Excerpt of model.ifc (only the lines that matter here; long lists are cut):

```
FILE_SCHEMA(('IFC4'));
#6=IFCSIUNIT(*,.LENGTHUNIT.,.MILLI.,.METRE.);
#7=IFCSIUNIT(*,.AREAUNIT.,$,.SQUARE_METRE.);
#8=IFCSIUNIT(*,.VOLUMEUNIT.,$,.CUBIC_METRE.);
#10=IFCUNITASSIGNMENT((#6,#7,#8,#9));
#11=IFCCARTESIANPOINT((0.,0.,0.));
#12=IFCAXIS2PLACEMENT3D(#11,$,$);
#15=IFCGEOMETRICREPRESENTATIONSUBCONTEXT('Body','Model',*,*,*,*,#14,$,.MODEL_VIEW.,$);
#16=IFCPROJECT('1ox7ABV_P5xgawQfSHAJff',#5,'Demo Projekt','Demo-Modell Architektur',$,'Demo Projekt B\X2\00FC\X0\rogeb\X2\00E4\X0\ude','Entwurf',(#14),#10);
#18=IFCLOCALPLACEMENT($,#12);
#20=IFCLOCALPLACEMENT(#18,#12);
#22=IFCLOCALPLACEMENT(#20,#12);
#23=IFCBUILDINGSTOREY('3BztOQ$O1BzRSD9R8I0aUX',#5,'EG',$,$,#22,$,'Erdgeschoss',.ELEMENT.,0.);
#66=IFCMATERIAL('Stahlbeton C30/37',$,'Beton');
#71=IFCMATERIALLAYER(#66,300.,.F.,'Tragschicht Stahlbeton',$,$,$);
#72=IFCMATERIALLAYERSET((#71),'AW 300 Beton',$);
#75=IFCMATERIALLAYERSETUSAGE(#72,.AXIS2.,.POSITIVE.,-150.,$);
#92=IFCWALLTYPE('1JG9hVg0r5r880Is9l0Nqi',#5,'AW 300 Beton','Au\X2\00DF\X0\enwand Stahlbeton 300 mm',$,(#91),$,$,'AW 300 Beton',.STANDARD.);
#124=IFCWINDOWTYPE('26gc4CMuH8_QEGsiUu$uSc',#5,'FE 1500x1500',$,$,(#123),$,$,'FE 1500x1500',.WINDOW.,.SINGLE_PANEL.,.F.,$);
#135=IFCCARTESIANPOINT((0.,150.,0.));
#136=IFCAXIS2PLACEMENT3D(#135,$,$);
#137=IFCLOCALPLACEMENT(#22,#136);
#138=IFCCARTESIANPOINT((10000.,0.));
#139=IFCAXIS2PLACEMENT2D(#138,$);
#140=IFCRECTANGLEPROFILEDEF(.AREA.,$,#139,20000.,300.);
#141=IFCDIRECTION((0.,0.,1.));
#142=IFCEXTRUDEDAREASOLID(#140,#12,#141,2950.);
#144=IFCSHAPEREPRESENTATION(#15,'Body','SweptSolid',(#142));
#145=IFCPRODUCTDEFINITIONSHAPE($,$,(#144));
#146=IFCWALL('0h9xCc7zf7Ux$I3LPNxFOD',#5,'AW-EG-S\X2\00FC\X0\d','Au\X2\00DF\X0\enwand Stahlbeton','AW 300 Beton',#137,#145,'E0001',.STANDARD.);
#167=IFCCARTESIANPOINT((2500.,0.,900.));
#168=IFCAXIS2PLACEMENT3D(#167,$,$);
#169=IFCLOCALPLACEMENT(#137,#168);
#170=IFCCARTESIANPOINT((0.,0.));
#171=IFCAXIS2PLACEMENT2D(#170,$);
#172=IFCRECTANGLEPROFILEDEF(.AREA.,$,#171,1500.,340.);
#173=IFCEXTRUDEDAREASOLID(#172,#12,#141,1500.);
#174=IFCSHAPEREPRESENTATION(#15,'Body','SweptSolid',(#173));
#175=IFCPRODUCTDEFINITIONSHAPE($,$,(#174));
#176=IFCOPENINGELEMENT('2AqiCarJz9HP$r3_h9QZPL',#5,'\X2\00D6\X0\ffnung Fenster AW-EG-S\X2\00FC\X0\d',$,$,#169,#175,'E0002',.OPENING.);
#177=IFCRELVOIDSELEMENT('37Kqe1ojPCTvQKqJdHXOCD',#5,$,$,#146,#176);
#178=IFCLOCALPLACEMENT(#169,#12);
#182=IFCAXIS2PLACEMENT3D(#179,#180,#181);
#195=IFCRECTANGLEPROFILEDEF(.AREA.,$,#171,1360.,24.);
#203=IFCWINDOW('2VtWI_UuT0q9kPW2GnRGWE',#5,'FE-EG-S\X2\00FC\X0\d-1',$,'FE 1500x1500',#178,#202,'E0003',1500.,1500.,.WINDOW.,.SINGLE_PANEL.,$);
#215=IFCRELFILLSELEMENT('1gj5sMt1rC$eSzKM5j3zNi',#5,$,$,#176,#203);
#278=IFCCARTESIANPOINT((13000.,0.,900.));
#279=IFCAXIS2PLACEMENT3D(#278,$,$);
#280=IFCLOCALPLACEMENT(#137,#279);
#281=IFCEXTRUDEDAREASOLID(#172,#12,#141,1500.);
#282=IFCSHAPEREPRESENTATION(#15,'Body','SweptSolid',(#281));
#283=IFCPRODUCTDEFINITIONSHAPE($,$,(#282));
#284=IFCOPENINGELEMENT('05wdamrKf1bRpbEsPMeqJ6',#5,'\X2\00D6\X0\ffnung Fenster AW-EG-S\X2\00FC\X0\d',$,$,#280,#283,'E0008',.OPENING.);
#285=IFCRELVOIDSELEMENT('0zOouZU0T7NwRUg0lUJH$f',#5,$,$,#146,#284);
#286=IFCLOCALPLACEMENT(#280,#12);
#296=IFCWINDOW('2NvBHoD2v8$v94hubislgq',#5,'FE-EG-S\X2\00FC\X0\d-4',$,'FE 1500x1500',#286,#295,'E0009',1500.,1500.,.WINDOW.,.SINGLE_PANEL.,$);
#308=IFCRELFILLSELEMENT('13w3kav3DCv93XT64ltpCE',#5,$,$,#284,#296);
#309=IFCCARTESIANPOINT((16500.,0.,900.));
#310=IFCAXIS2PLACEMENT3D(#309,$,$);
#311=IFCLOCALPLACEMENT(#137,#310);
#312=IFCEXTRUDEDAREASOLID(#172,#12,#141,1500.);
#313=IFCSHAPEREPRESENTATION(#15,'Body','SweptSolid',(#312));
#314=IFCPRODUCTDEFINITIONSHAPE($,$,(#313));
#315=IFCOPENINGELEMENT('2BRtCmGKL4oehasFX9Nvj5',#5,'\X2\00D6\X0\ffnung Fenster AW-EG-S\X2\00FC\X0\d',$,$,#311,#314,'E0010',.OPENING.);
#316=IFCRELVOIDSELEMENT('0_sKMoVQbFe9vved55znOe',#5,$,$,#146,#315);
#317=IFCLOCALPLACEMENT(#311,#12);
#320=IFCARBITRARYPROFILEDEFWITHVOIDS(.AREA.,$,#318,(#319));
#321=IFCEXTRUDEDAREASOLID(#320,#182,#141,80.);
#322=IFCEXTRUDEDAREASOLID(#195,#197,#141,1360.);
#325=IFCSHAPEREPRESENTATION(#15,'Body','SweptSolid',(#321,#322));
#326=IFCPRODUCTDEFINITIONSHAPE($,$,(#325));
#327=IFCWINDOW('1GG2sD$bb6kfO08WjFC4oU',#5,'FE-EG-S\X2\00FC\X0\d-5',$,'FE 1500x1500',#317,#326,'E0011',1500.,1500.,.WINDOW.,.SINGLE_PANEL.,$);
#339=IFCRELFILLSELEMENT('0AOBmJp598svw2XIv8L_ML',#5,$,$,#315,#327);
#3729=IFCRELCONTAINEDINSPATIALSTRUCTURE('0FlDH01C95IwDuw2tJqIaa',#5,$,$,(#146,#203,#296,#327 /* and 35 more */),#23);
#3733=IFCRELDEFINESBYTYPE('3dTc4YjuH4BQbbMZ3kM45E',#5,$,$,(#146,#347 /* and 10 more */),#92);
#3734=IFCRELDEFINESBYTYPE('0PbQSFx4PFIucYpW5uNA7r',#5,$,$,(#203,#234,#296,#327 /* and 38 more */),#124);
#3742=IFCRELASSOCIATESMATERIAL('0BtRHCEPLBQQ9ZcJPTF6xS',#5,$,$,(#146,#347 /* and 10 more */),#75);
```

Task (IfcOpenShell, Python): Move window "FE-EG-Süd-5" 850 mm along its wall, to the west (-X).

```python
import ifcopenshell
import ifcopenshell.api.geometry
import ifcopenshell.util.placement
import ifcopenshell.util.unit

model = ifcopenshell.open("model.ifc")
unit_scale = ifcopenshell.util.unit.calculate_unit_scale(model)

window = model.by_id(327)
opening = window.FillsVoids[0].RelatingOpeningElement
wall = opening.VoidsElements[0].RelatingBuildingElement

wall_matrix = ifcopenshell.util.placement.get_local_placement(wall.ObjectPlacement)
shift = wall_matrix[:3, 0] * -0.85 / unit_scale
before = ifcopenshell.util.placement.get_local_placement(window.ObjectPlacement)[:3, 3].copy()

# The window is placed relative to its opening, so it follows when the opening moves.
matrix = ifcopenshell.util.placement.get_local_placement(opening.ObjectPlacement)
matrix[:3, 3] += shift
ifcopenshell.api.geometry.edit_object_placement(
    model, product=opening, matrix=matrix, is_si=False, should_transform_children=True
)

after = ifcopenshell.util.placement.get_local_placement(window.ObjectPlacement)[:3, 3]
print("window moved by", (after - before).round(3) + 0.0)

model.write("model-out.ifc")
```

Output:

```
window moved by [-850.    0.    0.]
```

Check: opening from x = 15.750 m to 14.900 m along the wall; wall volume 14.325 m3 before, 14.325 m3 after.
